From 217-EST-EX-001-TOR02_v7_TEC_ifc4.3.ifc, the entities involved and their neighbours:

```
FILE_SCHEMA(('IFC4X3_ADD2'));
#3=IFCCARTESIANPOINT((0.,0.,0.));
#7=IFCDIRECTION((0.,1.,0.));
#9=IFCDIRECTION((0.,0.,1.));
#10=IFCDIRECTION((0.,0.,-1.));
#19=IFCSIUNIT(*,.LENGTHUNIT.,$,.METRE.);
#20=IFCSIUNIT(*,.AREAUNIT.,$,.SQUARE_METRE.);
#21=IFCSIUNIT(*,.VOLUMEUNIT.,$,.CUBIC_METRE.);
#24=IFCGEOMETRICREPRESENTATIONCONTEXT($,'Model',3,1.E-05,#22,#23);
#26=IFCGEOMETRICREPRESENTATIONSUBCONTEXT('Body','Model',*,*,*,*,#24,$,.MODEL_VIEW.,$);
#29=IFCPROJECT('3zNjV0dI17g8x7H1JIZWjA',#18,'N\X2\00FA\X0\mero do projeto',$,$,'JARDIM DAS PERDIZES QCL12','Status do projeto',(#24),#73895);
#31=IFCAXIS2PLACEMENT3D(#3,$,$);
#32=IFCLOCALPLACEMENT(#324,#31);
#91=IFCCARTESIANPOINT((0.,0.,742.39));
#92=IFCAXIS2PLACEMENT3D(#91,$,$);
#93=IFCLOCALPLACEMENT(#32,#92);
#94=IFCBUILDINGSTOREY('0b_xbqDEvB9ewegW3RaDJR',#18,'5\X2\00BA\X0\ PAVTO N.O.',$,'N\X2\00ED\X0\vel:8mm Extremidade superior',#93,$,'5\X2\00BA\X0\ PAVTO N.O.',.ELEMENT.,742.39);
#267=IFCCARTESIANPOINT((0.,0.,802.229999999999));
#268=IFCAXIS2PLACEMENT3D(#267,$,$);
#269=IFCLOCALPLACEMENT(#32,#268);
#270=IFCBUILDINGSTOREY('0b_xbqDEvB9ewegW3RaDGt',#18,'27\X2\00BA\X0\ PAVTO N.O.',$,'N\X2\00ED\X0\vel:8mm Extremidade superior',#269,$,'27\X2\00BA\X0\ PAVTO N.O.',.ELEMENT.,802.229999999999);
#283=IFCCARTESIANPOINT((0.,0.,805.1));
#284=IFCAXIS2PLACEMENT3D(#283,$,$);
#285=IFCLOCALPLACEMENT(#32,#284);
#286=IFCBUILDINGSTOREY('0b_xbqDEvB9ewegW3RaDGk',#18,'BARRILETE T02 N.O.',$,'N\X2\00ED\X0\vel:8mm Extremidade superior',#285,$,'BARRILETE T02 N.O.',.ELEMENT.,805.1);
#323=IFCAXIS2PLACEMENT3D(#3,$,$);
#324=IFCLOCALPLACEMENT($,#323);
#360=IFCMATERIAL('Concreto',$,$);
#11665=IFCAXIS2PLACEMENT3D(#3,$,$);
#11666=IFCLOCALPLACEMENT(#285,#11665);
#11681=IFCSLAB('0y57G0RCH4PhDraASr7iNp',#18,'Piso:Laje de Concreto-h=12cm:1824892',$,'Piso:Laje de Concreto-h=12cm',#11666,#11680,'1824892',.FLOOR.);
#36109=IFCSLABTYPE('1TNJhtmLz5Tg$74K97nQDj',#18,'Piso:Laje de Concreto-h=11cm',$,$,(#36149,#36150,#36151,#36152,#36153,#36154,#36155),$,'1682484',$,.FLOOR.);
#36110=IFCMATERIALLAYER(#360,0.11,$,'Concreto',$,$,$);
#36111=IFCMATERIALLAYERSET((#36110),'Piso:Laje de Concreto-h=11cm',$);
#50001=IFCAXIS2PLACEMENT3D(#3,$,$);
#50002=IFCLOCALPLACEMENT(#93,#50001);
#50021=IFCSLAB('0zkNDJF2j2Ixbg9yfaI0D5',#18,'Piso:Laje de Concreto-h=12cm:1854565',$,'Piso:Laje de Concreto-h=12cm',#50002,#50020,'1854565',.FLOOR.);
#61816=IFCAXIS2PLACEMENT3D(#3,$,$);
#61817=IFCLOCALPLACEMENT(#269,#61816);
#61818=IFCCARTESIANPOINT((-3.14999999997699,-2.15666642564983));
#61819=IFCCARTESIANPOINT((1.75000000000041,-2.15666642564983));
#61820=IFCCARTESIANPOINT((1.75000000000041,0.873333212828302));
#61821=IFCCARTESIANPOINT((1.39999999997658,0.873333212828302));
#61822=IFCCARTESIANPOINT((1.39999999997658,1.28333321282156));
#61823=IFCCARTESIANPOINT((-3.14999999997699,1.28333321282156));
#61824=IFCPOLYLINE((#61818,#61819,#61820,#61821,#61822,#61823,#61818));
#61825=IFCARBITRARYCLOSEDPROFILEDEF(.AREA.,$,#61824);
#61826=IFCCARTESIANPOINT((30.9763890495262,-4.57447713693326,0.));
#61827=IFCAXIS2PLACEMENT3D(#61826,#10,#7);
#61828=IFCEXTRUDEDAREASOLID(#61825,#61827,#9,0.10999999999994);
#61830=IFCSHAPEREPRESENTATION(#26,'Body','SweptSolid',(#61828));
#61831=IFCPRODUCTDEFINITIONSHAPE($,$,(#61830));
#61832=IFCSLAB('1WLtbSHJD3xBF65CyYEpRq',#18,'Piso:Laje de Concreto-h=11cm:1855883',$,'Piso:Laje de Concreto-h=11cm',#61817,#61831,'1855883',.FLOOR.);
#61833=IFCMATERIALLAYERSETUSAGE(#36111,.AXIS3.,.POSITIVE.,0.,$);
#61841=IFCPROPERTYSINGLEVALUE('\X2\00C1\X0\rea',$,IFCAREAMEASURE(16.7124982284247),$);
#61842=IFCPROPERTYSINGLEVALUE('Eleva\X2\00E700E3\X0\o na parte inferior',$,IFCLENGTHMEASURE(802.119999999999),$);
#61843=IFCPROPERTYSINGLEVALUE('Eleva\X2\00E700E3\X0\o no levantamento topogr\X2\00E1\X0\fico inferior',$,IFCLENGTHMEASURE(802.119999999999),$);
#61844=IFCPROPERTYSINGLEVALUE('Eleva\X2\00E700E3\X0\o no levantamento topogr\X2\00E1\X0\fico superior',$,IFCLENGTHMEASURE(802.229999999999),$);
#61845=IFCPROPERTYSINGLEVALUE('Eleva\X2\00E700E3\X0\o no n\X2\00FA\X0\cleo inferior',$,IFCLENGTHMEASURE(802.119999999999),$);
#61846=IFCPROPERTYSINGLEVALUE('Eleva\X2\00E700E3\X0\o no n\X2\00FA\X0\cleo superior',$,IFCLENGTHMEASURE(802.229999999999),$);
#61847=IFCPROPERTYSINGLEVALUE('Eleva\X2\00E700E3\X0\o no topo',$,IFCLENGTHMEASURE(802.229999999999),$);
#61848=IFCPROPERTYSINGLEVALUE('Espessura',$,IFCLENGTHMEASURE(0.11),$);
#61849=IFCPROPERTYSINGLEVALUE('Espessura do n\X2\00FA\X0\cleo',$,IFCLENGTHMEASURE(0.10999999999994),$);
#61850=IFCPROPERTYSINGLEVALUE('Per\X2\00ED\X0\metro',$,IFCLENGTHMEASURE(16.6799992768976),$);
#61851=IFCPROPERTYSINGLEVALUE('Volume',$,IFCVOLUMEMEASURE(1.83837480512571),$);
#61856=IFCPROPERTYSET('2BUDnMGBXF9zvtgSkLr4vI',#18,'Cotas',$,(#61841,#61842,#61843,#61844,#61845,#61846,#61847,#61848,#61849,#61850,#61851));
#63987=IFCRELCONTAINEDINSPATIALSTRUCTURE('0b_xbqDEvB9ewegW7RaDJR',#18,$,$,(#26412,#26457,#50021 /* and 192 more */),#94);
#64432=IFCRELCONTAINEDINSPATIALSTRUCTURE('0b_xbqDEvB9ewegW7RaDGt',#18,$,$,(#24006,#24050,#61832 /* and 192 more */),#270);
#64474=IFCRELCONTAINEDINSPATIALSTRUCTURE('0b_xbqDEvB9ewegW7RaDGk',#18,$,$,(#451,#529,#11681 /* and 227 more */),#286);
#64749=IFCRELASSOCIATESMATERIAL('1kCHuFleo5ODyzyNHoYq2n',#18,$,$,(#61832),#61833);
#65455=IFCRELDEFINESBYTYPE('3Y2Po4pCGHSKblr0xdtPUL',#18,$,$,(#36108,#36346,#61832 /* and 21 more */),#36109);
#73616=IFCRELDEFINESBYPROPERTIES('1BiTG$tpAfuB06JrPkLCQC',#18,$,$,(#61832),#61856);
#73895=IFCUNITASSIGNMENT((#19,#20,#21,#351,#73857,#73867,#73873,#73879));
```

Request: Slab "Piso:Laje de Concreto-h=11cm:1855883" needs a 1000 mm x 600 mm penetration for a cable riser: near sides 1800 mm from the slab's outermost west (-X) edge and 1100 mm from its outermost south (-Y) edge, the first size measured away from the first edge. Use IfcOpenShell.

```python
import numpy as np
import ifcopenshell
import ifcopenshell.api.feature
import ifcopenshell.api.geometry
import ifcopenshell.api.pset
import ifcopenshell.api.root
import ifcopenshell.geom
import ifcopenshell.util.element
import ifcopenshell.util.placement
import ifcopenshell.util.representation
import ifcopenshell.util.shape
import ifcopenshell.util.unit

model = ifcopenshell.open("217-EST-EX-001-TOR02_v7_TEC_ifc4.3.ifc")
unit_scale = ifcopenshell.util.unit.calculate_unit_scale(model)
area_scale = ifcopenshell.util.unit.calculate_unit_scale(model, "AREAUNIT")
volume_scale = ifcopenshell.util.unit.calculate_unit_scale(model, "VOLUMEUNIT")
settings = ifcopenshell.geom.settings()


def volume(element):
    """Net volume in cubic metres, openings subtracted."""
    shape = ifcopenshell.geom.create_shape(settings, element)
    return ifcopenshell.util.shape.get_volume(shape.geometry)


slab = model.by_guid("1WLtbSHJD3xBF65CyYEpRq")
before = volume(slab)

# Extent in the slab's own axes, in metres. The edges named are its -X and -Y sides.
slab_shape = ifcopenshell.geom.create_shape(settings, slab)
vertices = ifcopenshell.util.shape.get_vertices(slab_shape.geometry)
x_min, y_min, bottom = vertices.min(axis=0)
top = vertices[:, 2].max()

opening = ifcopenshell.api.root.create_entity(model, ifc_class="IfcOpeningElement", name="Cable riser opening", predefined_type="OPENING")
context = ifcopenshell.util.representation.get_context(model, "Model", "Body", "MODEL_VIEW")
width, depth = 1, 0.6
outline = [(0.0, 0.0), (width, 0.0), (width, depth), (0.0, depth), (0.0, 0.0)]
# Overshoot both faces by 50 mm so the cut is clean.
shape = ifcopenshell.api.geometry.add_slab_representation(
    model, context=context, depth=top - bottom + 0.1, polyline=outline
)
ifcopenshell.api.geometry.assign_representation(model, product=opening, representation=shape)

matrix = ifcopenshell.util.placement.get_local_placement(slab.ObjectPlacement)
matrix[:, 3] = matrix @ np.append(np.array([x_min + 1.8, y_min + 1.1, bottom - 0.05]) / unit_scale, 1.0)
ifcopenshell.api.geometry.edit_object_placement(model, product=opening, matrix=matrix, is_si=False)
ifcopenshell.api.feature.add_feature(model, feature=opening, element=slab)

after = volume(slab)

# Update the slab's stored quantities.
pset = model.by_id(ifcopenshell.util.element.get_pset(slab, "Cotas", should_inherit=False)["id"])
ifcopenshell.api.pset.edit_pset(model, pset=pset, properties={
    "Área": model.create_entity("IfcAreaMeasure", after / (top - bottom) / area_scale),
    "Volume": model.create_entity("IfcVolumeMeasure", after / volume_scale),
})

print(f"slab volume {before:.3f} -> {after:.3f} m3")

model.write("217-EST-EX-001-TOR02_v7_TEC_ifc4.3_edited.ifc")
```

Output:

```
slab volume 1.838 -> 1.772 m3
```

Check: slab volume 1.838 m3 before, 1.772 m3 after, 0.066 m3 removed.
